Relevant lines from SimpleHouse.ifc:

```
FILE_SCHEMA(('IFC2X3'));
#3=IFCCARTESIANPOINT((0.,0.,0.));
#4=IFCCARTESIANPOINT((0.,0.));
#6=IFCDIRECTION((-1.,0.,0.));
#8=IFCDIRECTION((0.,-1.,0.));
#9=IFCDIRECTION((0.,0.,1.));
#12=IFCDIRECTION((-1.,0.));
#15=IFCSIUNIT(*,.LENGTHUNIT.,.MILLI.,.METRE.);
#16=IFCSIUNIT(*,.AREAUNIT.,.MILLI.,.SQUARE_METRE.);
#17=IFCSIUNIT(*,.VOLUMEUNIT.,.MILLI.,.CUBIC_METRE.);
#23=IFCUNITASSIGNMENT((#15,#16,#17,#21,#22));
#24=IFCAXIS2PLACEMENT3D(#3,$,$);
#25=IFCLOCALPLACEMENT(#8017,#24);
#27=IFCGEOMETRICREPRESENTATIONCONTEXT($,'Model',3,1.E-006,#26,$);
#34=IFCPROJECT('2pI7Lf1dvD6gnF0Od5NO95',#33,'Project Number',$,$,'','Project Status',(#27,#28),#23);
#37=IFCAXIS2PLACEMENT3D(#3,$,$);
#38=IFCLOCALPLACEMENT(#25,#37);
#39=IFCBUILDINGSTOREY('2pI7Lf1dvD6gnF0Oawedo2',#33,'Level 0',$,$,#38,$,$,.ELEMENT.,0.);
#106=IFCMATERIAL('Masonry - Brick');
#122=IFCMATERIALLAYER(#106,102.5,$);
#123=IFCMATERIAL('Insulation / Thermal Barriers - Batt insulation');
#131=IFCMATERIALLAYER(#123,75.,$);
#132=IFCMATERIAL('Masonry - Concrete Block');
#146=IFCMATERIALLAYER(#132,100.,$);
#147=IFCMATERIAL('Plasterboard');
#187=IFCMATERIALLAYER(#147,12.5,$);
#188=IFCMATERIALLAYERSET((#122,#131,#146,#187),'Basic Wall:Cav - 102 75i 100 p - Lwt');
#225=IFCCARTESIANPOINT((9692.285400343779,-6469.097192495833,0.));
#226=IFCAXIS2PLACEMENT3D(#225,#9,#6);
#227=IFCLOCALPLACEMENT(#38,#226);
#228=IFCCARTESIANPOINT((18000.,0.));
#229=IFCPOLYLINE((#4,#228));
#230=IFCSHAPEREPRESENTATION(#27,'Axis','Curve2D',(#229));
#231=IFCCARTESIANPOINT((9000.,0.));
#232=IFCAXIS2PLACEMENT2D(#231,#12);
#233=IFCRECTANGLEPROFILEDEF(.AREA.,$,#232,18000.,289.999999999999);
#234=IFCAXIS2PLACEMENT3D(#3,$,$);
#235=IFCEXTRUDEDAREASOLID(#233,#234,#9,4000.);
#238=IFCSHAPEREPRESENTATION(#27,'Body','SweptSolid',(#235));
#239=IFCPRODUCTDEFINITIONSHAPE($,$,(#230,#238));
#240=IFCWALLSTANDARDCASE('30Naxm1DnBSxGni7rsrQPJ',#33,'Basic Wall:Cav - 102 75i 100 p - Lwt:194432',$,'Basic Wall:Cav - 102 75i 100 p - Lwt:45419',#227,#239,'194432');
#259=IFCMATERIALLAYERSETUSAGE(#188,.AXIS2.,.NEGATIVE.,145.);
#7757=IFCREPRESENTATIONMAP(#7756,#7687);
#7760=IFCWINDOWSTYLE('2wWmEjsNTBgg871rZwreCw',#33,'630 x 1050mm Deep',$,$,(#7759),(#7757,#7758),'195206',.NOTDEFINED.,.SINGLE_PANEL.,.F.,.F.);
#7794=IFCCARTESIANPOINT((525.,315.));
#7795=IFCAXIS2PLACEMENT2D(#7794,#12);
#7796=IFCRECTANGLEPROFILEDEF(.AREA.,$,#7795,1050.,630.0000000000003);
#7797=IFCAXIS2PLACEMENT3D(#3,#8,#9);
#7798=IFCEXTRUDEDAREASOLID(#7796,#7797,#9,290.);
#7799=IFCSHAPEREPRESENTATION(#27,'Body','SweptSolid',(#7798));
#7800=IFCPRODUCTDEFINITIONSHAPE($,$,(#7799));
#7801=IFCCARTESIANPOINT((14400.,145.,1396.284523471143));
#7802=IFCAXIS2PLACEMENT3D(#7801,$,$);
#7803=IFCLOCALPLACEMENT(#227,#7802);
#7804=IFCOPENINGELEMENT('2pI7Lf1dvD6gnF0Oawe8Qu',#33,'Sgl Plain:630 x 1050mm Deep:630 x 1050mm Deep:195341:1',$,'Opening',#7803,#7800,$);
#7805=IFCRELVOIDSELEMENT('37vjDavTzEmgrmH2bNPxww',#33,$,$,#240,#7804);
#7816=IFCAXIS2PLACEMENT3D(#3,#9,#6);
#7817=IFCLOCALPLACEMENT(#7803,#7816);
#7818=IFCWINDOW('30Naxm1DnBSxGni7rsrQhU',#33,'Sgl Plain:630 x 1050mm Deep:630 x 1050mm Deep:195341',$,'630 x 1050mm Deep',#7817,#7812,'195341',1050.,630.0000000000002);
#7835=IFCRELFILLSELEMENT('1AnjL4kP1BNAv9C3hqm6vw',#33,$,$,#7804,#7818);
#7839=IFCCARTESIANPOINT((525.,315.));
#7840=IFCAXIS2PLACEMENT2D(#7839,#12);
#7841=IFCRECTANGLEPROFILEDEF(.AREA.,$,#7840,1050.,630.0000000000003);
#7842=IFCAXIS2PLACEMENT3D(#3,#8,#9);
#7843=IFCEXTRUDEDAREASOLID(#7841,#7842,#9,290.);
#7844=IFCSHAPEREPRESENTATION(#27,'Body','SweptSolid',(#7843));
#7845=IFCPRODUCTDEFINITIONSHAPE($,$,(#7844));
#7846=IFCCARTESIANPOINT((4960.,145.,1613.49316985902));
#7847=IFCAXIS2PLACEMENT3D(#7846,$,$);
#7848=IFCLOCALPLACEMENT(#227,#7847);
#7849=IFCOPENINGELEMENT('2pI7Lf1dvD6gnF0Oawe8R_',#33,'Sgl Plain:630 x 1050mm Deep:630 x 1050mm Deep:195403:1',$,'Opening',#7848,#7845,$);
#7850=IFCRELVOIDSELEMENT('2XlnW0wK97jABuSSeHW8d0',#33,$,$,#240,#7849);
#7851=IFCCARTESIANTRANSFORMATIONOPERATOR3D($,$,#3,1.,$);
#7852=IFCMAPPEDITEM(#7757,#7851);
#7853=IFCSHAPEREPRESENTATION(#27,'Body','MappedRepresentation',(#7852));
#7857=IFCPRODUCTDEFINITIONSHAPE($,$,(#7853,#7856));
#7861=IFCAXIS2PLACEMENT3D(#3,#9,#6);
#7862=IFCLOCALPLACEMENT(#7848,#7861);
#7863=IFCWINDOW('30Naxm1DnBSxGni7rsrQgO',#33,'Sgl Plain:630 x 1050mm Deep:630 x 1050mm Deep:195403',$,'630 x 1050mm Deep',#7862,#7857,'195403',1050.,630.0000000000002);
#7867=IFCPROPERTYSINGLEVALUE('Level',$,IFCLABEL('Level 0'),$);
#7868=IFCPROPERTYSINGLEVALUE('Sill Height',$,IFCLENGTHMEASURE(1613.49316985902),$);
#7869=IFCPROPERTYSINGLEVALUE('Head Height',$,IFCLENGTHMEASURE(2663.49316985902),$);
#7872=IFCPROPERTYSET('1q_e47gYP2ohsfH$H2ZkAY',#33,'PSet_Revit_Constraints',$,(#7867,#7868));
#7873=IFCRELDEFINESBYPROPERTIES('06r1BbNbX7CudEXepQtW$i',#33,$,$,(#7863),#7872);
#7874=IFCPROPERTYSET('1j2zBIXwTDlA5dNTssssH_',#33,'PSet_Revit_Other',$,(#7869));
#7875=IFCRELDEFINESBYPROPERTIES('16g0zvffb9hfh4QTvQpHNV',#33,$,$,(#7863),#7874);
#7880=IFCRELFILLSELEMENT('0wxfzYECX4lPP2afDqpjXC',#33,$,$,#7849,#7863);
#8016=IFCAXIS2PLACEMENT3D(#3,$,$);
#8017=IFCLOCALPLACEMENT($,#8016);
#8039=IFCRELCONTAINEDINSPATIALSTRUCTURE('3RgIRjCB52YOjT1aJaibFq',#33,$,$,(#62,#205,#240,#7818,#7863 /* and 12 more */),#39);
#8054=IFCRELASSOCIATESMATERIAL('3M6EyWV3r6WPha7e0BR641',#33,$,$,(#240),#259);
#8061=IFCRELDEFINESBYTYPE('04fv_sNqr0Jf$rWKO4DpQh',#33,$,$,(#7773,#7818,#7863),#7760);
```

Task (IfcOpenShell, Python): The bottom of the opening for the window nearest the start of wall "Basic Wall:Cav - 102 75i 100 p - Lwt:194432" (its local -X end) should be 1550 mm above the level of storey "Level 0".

```python
import numpy as np
import ifcopenshell
import ifcopenshell.api.geometry
import ifcopenshell.api.pset
import ifcopenshell.geom
import ifcopenshell.util.element
import ifcopenshell.util.placement
import ifcopenshell.util.shape
import ifcopenshell.util.unit

model = ifcopenshell.open("SimpleHouse.ifc")
unit_scale = ifcopenshell.util.unit.calculate_unit_scale(model)

window = model.by_guid("30Naxm1DnBSxGni7rsrQgO")
opening = window.FillsVoids[0].RelatingOpeningElement
storey = ifcopenshell.util.element.get_container(window, ifc_class="IfcBuildingStorey")
level = ifcopenshell.util.placement.get_local_placement(storey.ObjectPlacement)[2, 3]

# The opening's origin need not be at the sill, so measure its lowest point.
shape = ifcopenshell.geom.create_shape(ifcopenshell.geom.settings(), opening)
bottom = ifcopenshell.util.shape.get_shape_bottom_elevation(shape, shape.geometry) / unit_scale
dz = level + 1.55 / unit_scale - bottom

shift = np.array([0.0, 0.0, dz])
# The window is placed relative to its opening, so it follows when the opening moves.
matrix = ifcopenshell.util.placement.get_local_placement(opening.ObjectPlacement)
matrix[:3, 3] += shift
ifcopenshell.api.geometry.edit_object_placement(
    model, product=opening, matrix=matrix, is_si=False, should_transform_children=True
)

# Keep the stored heights in step.
pset = model.by_id(ifcopenshell.util.element.get_pset(window, "PSet_Revit_Constraints", should_inherit=False)["id"])
ifcopenshell.api.pset.edit_pset(model, pset=pset, properties={
    "Sill Height": model.create_entity("IfcLengthMeasure", ifcopenshell.util.element.get_pset(window, "PSet_Revit_Constraints", "Sill Height") + dz),
})
pset = model.by_id(ifcopenshell.util.element.get_pset(window, "PSet_Revit_Other", should_inherit=False)["id"])
ifcopenshell.api.pset.edit_pset(model, pset=pset, properties={
    "Head Height": model.create_entity("IfcLengthMeasure", ifcopenshell.util.element.get_pset(window, "PSet_Revit_Other", "Head Height") + dz),
})

print(f"moved by {dz * unit_scale:+.3f} m")

model.write("SimpleHouse_updated.ifc")
```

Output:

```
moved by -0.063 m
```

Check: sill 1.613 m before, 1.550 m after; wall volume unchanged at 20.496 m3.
